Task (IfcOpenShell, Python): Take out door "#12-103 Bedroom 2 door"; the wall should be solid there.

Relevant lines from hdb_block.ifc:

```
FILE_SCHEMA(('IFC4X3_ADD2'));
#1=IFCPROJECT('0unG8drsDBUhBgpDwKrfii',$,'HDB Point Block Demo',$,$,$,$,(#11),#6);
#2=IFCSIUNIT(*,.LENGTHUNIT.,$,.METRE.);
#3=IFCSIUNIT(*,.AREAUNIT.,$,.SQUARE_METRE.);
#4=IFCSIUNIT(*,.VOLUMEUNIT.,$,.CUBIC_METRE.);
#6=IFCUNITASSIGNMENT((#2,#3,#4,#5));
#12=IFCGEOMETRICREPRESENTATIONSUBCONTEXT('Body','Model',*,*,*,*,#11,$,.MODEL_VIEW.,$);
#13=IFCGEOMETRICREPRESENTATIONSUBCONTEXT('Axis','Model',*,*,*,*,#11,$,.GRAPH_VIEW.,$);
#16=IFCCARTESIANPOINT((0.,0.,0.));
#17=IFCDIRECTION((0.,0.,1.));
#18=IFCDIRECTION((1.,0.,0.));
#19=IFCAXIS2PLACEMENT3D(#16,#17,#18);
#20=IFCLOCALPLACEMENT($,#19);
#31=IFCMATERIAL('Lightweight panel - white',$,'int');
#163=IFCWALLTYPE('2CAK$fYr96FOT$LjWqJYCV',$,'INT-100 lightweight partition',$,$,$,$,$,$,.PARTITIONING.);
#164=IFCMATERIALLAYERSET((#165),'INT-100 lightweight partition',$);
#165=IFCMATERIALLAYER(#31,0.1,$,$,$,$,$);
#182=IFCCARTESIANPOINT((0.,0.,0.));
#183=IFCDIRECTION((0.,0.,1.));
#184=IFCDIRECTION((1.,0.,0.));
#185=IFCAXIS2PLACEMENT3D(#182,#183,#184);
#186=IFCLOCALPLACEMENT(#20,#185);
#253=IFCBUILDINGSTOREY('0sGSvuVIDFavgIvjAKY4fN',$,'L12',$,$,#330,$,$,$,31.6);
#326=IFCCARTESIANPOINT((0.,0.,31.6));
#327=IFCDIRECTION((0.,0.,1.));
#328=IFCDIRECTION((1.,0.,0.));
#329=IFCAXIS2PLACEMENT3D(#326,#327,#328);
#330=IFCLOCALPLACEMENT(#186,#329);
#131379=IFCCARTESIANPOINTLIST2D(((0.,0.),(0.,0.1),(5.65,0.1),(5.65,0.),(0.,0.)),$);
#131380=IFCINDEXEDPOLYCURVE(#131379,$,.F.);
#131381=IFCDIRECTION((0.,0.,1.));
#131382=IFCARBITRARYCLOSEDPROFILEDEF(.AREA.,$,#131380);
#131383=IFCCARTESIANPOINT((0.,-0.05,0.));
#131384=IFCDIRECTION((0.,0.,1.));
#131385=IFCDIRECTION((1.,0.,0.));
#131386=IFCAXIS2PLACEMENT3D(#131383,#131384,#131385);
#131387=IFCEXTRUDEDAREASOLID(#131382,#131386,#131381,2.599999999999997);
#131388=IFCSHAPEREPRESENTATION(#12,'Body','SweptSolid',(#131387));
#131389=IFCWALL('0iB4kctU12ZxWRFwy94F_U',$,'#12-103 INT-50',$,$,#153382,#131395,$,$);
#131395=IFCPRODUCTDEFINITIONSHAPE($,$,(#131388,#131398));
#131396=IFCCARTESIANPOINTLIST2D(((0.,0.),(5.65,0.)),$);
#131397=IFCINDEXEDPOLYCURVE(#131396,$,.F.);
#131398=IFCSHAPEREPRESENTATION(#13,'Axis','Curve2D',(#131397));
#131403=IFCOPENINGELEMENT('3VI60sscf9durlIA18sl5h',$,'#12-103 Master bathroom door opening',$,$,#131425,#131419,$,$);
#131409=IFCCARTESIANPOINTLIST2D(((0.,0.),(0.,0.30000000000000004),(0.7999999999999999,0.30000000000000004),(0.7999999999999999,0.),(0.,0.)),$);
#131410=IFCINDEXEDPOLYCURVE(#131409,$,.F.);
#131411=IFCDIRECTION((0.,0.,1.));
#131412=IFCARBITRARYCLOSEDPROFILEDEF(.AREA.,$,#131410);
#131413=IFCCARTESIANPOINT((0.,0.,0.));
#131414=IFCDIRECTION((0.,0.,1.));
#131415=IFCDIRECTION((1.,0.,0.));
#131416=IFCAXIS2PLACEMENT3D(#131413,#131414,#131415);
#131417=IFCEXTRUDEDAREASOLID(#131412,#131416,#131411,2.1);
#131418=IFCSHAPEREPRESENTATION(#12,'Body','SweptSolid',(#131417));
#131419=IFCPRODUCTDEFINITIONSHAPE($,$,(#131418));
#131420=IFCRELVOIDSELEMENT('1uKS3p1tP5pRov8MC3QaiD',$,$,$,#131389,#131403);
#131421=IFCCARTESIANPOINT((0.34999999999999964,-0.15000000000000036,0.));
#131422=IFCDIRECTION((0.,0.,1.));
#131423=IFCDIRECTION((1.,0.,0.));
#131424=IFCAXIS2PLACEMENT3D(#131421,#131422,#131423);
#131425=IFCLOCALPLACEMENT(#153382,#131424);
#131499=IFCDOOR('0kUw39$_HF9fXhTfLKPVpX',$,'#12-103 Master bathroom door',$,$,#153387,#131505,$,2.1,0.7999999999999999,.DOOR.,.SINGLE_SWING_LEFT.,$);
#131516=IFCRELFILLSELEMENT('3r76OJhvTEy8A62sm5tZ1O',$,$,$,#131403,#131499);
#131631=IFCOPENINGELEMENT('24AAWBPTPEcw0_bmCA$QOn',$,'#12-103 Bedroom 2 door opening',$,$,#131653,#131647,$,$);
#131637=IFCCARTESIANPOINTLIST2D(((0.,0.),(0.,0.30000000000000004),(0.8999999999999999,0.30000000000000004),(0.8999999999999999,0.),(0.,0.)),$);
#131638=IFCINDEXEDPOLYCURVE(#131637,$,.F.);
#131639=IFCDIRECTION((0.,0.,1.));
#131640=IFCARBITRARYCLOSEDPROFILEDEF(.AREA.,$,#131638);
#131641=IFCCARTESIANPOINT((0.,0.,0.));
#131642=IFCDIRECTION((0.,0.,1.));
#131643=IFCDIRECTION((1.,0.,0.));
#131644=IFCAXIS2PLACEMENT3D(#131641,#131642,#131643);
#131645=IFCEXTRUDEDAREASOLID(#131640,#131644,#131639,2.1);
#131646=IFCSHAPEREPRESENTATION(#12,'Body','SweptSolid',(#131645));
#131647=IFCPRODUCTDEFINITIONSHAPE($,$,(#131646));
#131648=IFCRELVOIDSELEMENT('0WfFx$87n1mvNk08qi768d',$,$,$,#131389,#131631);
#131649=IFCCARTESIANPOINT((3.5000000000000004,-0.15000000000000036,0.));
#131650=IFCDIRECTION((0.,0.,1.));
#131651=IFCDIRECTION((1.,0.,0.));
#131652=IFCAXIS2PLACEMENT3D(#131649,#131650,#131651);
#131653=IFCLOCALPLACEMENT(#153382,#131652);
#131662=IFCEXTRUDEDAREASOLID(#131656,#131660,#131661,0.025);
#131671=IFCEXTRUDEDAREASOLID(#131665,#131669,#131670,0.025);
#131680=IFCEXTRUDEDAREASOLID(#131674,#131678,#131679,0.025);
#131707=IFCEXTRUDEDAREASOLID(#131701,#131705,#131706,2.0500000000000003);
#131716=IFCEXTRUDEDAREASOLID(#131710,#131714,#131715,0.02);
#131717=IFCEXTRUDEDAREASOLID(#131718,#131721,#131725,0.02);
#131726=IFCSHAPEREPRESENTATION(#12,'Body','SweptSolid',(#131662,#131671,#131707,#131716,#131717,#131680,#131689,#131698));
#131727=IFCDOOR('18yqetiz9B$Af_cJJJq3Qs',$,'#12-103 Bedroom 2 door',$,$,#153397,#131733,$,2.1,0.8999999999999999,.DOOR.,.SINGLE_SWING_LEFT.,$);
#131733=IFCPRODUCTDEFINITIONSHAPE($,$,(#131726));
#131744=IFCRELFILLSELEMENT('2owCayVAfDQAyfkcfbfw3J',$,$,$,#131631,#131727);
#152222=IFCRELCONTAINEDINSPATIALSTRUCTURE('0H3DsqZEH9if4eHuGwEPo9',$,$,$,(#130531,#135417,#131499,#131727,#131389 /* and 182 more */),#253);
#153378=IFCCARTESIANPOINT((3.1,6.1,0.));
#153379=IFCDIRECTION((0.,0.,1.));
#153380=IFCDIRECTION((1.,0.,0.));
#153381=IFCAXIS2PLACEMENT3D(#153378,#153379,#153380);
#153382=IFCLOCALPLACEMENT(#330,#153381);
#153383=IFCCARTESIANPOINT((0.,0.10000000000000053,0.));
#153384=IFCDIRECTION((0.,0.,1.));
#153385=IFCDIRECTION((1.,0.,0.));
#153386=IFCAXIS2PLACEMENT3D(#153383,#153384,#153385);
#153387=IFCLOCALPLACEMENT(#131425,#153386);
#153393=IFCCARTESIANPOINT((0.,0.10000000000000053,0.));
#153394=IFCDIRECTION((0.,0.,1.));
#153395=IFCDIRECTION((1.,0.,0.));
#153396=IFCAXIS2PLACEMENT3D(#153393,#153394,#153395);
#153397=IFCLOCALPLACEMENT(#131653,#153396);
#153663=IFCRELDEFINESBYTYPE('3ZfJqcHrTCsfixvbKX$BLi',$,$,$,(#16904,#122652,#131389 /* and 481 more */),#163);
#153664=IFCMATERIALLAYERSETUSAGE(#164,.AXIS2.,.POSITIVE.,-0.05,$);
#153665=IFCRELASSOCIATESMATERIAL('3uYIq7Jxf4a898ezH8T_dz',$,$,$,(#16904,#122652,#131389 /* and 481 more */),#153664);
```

```python
import ifcopenshell
import ifcopenshell.api.feature
import ifcopenshell.api.root
import ifcopenshell.geom
import ifcopenshell.util.shape

model = ifcopenshell.open("hdb_block.ifc")
settings = ifcopenshell.geom.settings()


def volume(element):
    """Net volume in cubic metres, openings subtracted."""
    shape = ifcopenshell.geom.create_shape(settings, element)
    return ifcopenshell.util.shape.get_volume(shape.geometry)


door = model.by_id(131727)
opening = door.FillsVoids[0].RelatingOpeningElement
wall = opening.VoidsElements[0].RelatingBuildingElement
before = volume(wall)

ifcopenshell.api.root.remove_product(model, product=door)
ifcopenshell.api.feature.remove_feature(model, feature=opening)

after = volume(wall)

print(f"wall volume {before:.3f} -> {after:.3f} m3")

model.write("hdb_block_rev.ifc")
```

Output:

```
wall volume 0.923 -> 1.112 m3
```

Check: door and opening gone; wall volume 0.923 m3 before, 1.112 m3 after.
